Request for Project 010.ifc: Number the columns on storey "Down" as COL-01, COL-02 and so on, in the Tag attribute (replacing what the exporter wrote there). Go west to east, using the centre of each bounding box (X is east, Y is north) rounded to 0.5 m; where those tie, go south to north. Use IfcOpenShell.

First a look at what the model holds.

```python
import ifcopenshell
import ifcopenshell.util.element
import ifcopenshell.util.placement

model = ifcopenshell.open("Project 010.ifc")
print(model.schema)
storey = next(s for s in model.by_type("IfcBuildingStorey") if s.Name == "Down")
columns = [e for e in ifcopenshell.util.element.get_decomposition(storey) if e.is_a("IfcColumn")]
for e in sorted(columns, key=lambda e: e.id()):
    origin = ifcopenshell.util.placement.get_local_placement(e.ObjectPlacement)[:3, 3]
    print(e.id(), e.Tag, e.Name, origin.round(2) + 0.0, sep=" | ")
```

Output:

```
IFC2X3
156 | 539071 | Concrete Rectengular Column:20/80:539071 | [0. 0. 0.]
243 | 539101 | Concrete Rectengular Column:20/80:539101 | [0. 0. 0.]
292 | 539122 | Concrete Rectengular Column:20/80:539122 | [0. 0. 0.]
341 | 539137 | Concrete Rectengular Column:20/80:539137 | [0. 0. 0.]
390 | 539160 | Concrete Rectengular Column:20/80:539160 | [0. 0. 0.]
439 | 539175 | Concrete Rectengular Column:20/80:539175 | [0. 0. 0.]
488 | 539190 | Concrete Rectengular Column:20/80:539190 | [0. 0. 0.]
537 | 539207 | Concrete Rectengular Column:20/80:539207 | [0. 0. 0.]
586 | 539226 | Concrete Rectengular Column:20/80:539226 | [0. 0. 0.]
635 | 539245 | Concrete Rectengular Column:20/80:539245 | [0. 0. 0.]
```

```python
import ifcopenshell
import ifcopenshell.geom
import ifcopenshell.util.element
import ifcopenshell.util.shape

model = ifcopenshell.open("Project 010.ifc")
settings = ifcopenshell.geom.settings()
settings.set("use-world-coords", True)


def centre(element):
    shape = ifcopenshell.geom.create_shape(settings, element)
    return ifcopenshell.util.shape.get_bbox_centroid(shape.geometry)


storey = next(s for s in model.by_type("IfcBuildingStorey") if s.Name == "Down")
columns = [e for e in ifcopenshell.util.element.get_decomposition(storey) if e.is_a("IfcColumn")]

# Insertion points can sit at a corner or the storey origin, so sort by the geometry (in metres).
centres = {e: centre(e) for e in columns}
columns.sort(key=lambda e: (round(centres[e][0] / 0.5), centres[e][1]))

for i, e in enumerate(columns, start=1):
    number = f"COL-{i:02d}"
    e.Tag = number
    print(e.id(), number)

model.write("Project 010_edited.ifc")
```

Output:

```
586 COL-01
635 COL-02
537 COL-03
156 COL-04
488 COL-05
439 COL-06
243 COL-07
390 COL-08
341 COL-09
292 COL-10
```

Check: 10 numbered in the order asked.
